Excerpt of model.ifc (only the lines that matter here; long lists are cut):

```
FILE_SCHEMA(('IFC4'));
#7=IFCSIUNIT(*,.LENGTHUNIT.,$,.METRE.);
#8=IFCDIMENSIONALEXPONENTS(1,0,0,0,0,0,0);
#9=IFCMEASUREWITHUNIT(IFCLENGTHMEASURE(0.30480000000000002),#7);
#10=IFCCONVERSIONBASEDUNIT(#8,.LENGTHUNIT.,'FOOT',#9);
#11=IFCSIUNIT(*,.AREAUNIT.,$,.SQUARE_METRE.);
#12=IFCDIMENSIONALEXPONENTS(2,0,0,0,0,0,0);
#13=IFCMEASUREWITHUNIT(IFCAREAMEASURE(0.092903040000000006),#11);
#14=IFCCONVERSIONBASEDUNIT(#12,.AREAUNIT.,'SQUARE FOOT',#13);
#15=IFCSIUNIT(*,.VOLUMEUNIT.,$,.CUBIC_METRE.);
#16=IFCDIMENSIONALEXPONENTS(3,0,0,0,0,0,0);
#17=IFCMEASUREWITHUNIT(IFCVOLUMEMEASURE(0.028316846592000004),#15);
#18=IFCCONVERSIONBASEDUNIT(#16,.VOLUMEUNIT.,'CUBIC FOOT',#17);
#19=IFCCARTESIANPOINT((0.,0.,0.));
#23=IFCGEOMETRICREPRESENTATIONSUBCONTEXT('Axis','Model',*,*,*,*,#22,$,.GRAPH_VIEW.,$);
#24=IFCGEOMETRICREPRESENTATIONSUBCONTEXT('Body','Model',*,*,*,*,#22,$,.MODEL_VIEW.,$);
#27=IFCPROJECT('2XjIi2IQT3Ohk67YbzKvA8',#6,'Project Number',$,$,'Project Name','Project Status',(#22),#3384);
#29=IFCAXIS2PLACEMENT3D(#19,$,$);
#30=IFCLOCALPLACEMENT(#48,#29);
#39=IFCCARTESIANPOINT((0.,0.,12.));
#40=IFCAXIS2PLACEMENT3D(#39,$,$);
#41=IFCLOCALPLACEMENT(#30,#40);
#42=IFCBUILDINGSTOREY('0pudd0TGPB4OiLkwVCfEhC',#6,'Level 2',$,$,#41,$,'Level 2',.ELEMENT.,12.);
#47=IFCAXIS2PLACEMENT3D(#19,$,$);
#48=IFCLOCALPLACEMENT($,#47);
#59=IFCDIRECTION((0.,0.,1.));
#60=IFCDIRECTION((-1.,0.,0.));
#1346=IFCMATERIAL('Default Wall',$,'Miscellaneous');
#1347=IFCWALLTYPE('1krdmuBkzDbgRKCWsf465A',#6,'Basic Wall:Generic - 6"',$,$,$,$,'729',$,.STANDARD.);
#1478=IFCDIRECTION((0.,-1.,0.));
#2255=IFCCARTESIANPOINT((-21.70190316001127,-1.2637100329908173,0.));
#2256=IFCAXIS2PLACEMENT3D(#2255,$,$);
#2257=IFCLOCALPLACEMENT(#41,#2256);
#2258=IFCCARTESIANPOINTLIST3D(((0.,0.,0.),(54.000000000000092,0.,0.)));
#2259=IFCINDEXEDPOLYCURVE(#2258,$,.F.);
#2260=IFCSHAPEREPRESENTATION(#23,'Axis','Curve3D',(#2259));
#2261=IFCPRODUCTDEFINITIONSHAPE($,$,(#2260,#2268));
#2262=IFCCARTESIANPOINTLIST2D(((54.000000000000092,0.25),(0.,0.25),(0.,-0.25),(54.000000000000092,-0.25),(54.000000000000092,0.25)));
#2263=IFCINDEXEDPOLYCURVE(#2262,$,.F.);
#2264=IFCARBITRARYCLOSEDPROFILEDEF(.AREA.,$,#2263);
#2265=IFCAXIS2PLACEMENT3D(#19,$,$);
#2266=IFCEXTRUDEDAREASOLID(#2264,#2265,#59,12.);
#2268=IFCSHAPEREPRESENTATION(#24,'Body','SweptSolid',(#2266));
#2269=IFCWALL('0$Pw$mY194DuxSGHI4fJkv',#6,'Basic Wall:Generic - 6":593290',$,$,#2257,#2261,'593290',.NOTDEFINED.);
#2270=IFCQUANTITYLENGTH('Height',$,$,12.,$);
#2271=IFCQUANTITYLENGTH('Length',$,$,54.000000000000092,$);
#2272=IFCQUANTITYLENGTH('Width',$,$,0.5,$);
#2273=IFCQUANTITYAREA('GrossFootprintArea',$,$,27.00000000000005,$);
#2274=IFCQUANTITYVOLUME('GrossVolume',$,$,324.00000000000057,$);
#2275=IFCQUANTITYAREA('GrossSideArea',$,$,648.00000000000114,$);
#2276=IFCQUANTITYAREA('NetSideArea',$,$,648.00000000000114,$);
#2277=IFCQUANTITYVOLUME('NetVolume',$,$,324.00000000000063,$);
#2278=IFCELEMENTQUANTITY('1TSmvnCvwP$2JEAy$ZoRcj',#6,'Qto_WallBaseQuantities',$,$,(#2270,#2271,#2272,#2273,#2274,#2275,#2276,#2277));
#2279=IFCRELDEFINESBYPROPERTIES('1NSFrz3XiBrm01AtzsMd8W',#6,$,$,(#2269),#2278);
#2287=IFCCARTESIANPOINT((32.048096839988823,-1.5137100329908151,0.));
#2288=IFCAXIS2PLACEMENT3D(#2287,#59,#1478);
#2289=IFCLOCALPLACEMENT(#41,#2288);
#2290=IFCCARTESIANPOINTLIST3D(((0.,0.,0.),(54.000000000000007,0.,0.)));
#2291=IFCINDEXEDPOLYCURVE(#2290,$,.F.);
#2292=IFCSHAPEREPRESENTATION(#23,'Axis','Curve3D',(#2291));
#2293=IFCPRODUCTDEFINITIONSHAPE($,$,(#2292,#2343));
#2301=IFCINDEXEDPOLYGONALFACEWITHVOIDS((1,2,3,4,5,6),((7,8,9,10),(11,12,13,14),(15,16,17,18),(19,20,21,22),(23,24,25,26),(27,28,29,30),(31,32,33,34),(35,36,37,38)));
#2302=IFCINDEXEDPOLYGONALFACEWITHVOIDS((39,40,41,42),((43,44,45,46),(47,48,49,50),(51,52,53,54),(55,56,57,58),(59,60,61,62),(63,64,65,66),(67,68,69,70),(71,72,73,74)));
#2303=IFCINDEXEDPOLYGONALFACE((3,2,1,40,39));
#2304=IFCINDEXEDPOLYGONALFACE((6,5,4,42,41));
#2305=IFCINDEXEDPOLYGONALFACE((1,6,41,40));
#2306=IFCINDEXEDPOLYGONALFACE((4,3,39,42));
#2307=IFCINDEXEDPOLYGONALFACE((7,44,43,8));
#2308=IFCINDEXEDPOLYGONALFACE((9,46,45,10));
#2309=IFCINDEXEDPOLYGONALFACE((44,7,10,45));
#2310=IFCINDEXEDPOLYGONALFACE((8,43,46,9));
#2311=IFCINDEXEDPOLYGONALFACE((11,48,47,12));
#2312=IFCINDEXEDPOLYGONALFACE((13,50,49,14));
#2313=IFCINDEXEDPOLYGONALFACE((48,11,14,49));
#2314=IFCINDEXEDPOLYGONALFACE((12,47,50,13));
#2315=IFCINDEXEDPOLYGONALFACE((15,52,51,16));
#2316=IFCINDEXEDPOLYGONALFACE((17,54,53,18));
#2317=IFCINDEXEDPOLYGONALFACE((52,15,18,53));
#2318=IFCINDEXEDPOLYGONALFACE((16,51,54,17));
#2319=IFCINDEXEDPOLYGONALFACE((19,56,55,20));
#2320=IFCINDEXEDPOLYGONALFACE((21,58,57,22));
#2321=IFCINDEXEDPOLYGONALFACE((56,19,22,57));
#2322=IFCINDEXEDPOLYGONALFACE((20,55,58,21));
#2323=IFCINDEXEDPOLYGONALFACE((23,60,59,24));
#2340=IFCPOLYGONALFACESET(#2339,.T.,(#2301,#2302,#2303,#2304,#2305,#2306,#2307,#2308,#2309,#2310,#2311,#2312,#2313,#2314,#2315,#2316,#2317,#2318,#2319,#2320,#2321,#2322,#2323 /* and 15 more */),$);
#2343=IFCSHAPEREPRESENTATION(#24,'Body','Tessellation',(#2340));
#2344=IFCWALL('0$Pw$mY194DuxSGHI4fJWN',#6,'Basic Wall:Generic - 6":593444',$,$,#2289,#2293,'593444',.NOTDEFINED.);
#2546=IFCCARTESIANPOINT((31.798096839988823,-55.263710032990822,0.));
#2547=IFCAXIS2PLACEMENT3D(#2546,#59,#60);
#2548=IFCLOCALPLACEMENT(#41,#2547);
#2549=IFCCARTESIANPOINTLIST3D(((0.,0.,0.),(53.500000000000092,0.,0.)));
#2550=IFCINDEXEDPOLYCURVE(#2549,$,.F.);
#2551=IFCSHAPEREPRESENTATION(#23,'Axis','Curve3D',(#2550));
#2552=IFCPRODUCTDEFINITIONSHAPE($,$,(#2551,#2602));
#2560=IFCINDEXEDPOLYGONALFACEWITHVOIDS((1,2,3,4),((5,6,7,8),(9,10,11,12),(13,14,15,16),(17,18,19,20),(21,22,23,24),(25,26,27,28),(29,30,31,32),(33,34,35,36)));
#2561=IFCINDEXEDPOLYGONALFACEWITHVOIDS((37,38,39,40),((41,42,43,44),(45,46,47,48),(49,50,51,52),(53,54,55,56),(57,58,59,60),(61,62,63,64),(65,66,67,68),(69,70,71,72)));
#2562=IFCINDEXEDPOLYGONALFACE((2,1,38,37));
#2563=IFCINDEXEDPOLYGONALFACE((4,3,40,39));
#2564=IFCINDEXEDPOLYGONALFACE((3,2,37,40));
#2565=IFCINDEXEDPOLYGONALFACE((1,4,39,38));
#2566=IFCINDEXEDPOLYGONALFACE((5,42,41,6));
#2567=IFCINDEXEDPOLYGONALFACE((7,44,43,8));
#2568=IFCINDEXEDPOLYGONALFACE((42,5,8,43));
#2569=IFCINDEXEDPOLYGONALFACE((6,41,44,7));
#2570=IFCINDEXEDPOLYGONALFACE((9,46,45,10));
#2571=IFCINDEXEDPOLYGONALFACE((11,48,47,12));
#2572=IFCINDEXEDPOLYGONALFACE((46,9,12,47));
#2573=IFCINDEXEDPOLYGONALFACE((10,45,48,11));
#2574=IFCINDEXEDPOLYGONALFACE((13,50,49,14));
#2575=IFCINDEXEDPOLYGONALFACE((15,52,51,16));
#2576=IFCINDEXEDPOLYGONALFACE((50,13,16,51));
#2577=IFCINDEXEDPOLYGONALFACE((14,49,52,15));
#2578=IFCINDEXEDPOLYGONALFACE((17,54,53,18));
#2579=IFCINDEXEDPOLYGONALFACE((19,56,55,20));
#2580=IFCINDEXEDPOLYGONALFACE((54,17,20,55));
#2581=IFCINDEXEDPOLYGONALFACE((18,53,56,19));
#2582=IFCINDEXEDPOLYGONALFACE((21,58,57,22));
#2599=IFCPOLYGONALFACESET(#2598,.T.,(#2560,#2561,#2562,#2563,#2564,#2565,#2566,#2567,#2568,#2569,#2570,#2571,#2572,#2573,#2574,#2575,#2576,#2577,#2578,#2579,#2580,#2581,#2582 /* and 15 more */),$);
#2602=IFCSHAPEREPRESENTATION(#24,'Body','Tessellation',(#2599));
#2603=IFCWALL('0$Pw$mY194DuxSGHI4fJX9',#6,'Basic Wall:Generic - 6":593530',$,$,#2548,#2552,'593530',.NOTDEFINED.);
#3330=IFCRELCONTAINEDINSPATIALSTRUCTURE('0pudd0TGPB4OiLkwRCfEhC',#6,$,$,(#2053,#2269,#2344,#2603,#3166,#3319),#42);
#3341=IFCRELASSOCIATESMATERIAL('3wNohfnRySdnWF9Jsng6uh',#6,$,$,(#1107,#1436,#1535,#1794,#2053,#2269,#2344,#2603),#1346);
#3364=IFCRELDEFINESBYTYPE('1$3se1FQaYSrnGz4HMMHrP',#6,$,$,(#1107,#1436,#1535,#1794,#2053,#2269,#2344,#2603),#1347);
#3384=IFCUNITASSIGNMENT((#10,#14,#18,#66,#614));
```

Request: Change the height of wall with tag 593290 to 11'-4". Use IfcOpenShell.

```python
import ifcopenshell
import ifcopenshell.api.pset
import ifcopenshell.geom
import ifcopenshell.util.element
import ifcopenshell.util.representation
import ifcopenshell.util.shape
import ifcopenshell.util.unit

model = ifcopenshell.open("model.ifc")
unit_scale = ifcopenshell.util.unit.calculate_unit_scale(model)
area_scale = ifcopenshell.util.unit.calculate_unit_scale(model, "AREAUNIT")
volume_scale = ifcopenshell.util.unit.calculate_unit_scale(model, "VOLUMEUNIT")
settings = ifcopenshell.geom.settings()


def volume(element):
    """Net volume in cubic metres, openings subtracted."""
    shape = ifcopenshell.geom.create_shape(settings, element)
    return ifcopenshell.util.shape.get_volume(shape.geometry)


wall = model.by_id(2269)
before = volume(wall)

body = ifcopenshell.util.representation.get_representation(wall, "Model", "Body")
solid = body.Items[0]
old_height = solid.Depth
solid.Depth = 136 * 0.0254 / unit_scale
after = volume(wall)
thickness = 0.1524  # wall thickness in metres

# Update the stored height, areas and volumes.
qto = model.by_id(ifcopenshell.util.element.get_pset(wall, "Qto_WallBaseQuantities", should_inherit=False)["id"])
ifcopenshell.api.pset.edit_qto(model, qto=qto, properties={
    "Height": solid.Depth,
    "GrossVolume": ifcopenshell.util.element.get_pset(wall, "Qto_WallBaseQuantities", "GrossVolume") * solid.Depth / old_height,
    "GrossSideArea": ifcopenshell.util.element.get_pset(wall, "Qto_WallBaseQuantities", "GrossSideArea") * solid.Depth / old_height,
    "NetSideArea": after / thickness / area_scale,
    "NetVolume": after / volume_scale,
})

print(f"height {old_height:g} -> {solid.Depth:g}, volume {before:.3f} -> {after:.3f} m3")

model.write("model_rev.ifc")
```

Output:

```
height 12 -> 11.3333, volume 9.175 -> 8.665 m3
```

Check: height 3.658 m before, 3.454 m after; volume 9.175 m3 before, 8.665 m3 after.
